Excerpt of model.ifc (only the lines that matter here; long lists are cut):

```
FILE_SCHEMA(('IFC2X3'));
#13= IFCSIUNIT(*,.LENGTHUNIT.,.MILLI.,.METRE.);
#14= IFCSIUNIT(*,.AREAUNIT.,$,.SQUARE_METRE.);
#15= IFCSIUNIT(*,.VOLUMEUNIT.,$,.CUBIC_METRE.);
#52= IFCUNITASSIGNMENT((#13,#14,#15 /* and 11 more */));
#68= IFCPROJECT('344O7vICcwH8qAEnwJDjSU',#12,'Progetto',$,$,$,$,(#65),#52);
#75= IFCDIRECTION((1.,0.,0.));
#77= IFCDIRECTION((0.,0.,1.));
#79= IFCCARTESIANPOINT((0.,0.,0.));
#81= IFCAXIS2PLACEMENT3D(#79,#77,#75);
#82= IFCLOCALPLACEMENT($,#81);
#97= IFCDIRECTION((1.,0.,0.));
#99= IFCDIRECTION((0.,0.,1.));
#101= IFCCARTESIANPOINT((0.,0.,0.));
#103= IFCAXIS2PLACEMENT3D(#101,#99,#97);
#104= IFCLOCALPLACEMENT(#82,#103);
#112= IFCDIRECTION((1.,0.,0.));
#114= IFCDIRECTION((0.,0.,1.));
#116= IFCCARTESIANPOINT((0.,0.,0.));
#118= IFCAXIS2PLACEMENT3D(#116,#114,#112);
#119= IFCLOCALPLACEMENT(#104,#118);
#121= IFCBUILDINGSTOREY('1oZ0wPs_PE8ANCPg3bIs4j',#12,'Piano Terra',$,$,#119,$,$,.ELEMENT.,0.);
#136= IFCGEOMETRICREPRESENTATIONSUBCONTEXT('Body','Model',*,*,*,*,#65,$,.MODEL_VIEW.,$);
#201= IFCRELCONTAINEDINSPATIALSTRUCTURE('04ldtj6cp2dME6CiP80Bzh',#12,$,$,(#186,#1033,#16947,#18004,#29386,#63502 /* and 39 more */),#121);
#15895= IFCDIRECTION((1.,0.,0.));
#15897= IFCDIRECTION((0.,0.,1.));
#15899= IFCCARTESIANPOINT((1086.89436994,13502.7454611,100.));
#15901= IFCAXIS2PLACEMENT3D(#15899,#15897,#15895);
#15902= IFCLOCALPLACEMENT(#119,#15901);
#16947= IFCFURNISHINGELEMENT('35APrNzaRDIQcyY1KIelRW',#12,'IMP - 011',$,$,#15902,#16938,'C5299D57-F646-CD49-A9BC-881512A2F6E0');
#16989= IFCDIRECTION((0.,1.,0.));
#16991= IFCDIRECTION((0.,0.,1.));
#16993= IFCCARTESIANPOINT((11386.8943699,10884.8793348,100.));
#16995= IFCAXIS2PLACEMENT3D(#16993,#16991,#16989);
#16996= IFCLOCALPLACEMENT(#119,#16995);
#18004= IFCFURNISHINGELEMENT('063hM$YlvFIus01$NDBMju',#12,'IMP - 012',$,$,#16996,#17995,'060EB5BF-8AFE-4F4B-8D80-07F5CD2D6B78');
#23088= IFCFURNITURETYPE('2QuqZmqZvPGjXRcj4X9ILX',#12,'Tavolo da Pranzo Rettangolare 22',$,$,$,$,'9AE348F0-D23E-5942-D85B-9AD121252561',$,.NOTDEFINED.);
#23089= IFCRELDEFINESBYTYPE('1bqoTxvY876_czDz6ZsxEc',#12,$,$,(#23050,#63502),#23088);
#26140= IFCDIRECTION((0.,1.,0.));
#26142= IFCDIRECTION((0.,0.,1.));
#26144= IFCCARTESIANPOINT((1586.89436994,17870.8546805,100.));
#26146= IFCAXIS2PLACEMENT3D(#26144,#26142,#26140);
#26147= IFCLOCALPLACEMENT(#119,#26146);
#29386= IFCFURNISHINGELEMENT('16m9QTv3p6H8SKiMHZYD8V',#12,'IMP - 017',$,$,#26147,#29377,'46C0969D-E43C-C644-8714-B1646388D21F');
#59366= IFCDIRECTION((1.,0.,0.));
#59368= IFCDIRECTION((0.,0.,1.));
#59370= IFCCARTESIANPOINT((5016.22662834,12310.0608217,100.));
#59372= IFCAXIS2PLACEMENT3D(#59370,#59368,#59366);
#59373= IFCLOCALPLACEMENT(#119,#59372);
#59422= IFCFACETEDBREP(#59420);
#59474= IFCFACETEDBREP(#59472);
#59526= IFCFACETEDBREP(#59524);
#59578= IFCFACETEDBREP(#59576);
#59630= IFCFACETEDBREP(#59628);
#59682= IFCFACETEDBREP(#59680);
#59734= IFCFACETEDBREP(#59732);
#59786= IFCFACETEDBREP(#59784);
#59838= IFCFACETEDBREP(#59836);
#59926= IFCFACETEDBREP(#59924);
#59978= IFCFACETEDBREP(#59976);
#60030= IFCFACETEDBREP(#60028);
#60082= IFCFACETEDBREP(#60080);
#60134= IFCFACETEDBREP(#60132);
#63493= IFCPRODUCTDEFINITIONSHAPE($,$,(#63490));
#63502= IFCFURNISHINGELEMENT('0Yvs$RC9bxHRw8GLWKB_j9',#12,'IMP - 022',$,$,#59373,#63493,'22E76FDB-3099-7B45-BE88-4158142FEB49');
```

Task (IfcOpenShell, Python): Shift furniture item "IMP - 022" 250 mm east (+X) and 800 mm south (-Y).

```python
import ifcopenshell
import ifcopenshell.api.geometry
import ifcopenshell.util.placement
import ifcopenshell.util.unit

model = ifcopenshell.open("model.ifc")
unit_scale = ifcopenshell.util.unit.calculate_unit_scale(model)

item = model.by_guid("0Yvs$RC9bxHRw8GLWKB_j9")
matrix = ifcopenshell.util.placement.get_local_placement(item.ObjectPlacement)
matrix[0, 3] += 0.25 / unit_scale
matrix[1, 3] -= 0.8 / unit_scale
ifcopenshell.api.geometry.edit_object_placement(model, product=item, matrix=matrix, is_si=False)

print(ifcopenshell.util.placement.get_local_placement(item.ObjectPlacement).round(3) + 0.0)

model.write("model_edited.ifc")
```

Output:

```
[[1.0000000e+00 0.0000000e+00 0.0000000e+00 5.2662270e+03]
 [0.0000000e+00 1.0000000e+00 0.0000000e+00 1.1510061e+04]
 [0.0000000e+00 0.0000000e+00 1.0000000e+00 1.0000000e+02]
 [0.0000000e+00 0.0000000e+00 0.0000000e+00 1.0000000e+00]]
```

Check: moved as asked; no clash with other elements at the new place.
